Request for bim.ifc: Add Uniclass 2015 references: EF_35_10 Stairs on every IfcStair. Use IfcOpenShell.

First a look at what the model holds.

```python
import ifcopenshell

model = ifcopenshell.open("bim.ifc")
print(model.schema)
print("classifications:", [c.Name for c in model.by_type("IfcClassification")])
for ifc_class in ("IfcDoor", "IfcRoof", "IfcStair", "IfcWall", "IfcWindow"):
    print(ifc_class, len(model.by_type(ifc_class)))
```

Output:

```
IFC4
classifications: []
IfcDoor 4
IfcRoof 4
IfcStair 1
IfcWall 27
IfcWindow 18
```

```python
import ifcopenshell
import ifcopenshell.api.classification

model = ifcopenshell.open("bim.ifc")

system = ifcopenshell.api.classification.add_classification(model, classification="Uniclass 2015")

codes = {
    "IfcStair": ("EF_35_10", "Stairs"),
}
for ifc_class, (code, name) in codes.items():
    products = model.by_type(ifc_class)
    ifcopenshell.api.classification.add_reference(
        model, products=products, classification=system, identification=code, name=name
    )
    print(code, len(products))

model.write("bim_rev.ifc")
```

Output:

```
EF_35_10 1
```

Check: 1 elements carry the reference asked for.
